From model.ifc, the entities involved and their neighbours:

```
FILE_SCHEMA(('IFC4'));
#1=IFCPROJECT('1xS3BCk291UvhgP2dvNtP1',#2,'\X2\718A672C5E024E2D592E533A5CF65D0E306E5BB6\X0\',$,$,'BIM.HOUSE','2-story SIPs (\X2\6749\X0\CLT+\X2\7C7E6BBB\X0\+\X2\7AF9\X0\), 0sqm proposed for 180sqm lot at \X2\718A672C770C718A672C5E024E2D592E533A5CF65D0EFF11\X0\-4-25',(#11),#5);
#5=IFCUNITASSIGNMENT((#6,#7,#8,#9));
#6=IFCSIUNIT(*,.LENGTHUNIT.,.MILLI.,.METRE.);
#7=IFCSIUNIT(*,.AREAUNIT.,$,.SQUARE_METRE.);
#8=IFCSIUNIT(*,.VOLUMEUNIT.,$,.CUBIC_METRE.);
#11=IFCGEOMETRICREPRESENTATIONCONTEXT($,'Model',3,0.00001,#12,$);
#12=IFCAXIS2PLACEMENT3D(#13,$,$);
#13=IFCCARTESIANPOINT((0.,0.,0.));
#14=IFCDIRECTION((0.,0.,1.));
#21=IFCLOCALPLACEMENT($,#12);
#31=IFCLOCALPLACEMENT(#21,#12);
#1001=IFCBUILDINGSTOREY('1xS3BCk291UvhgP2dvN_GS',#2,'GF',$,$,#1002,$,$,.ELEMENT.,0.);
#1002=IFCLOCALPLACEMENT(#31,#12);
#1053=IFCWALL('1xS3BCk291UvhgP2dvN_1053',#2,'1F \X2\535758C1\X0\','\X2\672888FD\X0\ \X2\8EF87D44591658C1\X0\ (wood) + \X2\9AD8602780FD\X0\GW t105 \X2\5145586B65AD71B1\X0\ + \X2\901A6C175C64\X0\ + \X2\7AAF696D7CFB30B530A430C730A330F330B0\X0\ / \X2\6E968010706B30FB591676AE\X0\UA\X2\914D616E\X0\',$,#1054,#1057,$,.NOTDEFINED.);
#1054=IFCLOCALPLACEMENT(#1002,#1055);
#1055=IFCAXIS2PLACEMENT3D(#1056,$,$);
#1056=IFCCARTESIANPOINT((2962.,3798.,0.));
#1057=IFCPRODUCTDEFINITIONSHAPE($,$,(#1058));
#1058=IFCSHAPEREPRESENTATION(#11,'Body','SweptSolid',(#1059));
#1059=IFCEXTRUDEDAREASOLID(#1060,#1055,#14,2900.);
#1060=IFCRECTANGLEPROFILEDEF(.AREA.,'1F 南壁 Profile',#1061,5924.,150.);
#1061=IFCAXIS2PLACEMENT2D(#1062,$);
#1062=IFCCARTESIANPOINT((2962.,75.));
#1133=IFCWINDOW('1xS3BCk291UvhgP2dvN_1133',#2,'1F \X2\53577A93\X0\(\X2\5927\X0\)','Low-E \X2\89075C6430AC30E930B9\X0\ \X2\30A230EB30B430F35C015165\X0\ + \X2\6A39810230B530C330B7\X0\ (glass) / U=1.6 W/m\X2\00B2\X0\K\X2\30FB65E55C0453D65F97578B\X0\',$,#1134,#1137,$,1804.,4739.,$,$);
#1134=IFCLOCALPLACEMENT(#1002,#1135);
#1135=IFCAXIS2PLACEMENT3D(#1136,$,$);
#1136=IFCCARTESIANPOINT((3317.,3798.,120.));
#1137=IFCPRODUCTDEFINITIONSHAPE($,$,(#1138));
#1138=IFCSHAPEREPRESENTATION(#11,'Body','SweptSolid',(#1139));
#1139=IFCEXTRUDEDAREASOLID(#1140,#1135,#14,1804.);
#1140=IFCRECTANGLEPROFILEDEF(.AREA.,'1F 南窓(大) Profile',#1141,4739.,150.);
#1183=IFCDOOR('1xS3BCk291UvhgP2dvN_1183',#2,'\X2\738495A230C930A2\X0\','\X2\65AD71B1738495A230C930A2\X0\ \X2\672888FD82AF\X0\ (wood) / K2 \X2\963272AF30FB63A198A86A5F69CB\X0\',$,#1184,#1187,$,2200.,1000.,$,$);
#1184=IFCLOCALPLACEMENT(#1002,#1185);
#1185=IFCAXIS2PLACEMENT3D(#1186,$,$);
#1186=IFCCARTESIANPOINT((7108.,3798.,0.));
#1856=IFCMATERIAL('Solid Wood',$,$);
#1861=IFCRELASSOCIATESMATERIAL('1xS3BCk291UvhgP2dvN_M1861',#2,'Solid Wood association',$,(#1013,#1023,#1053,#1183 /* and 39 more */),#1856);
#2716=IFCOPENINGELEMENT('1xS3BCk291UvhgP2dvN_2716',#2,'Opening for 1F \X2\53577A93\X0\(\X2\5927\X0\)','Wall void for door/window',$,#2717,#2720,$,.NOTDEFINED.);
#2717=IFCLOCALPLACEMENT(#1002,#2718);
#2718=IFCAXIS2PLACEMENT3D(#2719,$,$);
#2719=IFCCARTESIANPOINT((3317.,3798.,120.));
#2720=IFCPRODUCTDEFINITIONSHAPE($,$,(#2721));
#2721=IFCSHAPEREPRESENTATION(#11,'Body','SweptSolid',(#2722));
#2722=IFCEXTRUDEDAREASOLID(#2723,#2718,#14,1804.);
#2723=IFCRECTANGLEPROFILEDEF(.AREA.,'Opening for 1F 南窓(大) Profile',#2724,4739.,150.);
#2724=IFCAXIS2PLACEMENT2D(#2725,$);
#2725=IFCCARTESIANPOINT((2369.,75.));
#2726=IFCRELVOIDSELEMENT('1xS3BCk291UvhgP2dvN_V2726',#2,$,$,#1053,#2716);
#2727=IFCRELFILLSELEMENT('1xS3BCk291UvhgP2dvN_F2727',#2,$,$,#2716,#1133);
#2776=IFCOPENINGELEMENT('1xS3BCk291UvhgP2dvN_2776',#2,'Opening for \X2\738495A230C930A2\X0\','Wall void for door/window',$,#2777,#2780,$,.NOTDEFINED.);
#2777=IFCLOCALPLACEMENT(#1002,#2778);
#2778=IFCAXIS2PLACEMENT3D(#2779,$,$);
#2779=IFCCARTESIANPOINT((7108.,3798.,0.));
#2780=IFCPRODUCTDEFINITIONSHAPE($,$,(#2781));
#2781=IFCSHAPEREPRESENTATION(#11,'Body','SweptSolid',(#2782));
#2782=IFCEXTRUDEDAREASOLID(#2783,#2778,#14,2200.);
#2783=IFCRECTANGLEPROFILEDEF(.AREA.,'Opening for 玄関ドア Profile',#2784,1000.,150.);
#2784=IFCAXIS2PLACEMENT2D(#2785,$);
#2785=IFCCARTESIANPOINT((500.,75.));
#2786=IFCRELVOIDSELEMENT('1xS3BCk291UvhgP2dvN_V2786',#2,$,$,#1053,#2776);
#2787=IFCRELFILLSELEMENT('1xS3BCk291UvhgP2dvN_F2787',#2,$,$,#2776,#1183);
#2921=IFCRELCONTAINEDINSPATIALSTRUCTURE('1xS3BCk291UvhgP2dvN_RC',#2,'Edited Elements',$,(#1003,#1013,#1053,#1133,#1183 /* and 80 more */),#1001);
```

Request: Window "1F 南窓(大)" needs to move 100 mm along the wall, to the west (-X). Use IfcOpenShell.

```python
import ifcopenshell
import ifcopenshell.api.geometry
import ifcopenshell.util.placement
import ifcopenshell.util.unit

model = ifcopenshell.open("model.ifc")
unit_scale = ifcopenshell.util.unit.calculate_unit_scale(model)

window = model.by_guid("1xS3BCk291UvhgP2dvN_1133")
opening = window.FillsVoids[0].RelatingOpeningElement
wall = opening.VoidsElements[0].RelatingBuildingElement

wall_matrix = ifcopenshell.util.placement.get_local_placement(wall.ObjectPlacement)
shift = wall_matrix[:3, 0] * -0.1 / unit_scale
before = ifcopenshell.util.placement.get_local_placement(window.ObjectPlacement)[:3, 3].copy()

# The window is not placed relative to its opening, so move both.
for product in (opening, window):
    matrix = ifcopenshell.util.placement.get_local_placement(product.ObjectPlacement)
    matrix[:3, 3] += shift
    ifcopenshell.api.geometry.edit_object_placement(model, product=product, matrix=matrix, is_si=False)

after = ifcopenshell.util.placement.get_local_placement(window.ObjectPlacement)[:3, 3]
print("window moved by", (after - before).round(3) + 0.0)

model.write("model-out.ifc")
```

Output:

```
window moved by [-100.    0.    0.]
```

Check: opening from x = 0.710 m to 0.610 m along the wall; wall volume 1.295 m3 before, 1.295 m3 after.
